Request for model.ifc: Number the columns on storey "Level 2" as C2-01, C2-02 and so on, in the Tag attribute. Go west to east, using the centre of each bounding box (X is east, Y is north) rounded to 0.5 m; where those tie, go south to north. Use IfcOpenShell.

First a look at what the model holds.

```python
import ifcopenshell
import ifcopenshell.util.element
import ifcopenshell.util.placement

model = ifcopenshell.open("model.ifc")
print(model.schema)
storey = next(s for s in model.by_type("IfcBuildingStorey") if s.Name == "Level 2")
columns = [e for e in ifcopenshell.util.element.get_decomposition(storey) if e.is_a("IfcColumn")]
for e in sorted(columns, key=lambda e: e.id()):
    origin = ifcopenshell.util.placement.get_local_placement(e.ObjectPlacement)[:3, 3]
    print(e.id(), e.Tag, e.Name, origin.round(2) + 0.0, sep=" | ")
```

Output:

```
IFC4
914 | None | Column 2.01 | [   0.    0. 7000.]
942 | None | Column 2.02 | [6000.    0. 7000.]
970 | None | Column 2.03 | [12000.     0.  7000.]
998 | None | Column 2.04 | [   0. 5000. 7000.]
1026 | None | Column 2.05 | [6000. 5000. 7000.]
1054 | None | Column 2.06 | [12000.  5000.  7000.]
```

```python
import ifcopenshell
import ifcopenshell.geom
import ifcopenshell.util.element
import ifcopenshell.util.shape

model = ifcopenshell.open("model.ifc")
settings = ifcopenshell.geom.settings()
settings.set("use-world-coords", True)


def centre(element):
    shape = ifcopenshell.geom.create_shape(settings, element)
    return ifcopenshell.util.shape.get_bbox_centroid(shape.geometry)


storey = next(s for s in model.by_type("IfcBuildingStorey") if s.Name == "Level 2")
columns = [e for e in ifcopenshell.util.element.get_decomposition(storey) if e.is_a("IfcColumn")]

# Insertion points can sit at a corner or the storey origin, so sort by the geometry (in metres).
centres = {e: centre(e) for e in columns}
columns.sort(key=lambda e: (round(centres[e][0] / 0.5), centres[e][1]))

for i, e in enumerate(columns, start=1):
    number = f"C2-{i:02d}"
    e.Tag = number
    print(e.id(), number)

model.write("model-out.ifc")
```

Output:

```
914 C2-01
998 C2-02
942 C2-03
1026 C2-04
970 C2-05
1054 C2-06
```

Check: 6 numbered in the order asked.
